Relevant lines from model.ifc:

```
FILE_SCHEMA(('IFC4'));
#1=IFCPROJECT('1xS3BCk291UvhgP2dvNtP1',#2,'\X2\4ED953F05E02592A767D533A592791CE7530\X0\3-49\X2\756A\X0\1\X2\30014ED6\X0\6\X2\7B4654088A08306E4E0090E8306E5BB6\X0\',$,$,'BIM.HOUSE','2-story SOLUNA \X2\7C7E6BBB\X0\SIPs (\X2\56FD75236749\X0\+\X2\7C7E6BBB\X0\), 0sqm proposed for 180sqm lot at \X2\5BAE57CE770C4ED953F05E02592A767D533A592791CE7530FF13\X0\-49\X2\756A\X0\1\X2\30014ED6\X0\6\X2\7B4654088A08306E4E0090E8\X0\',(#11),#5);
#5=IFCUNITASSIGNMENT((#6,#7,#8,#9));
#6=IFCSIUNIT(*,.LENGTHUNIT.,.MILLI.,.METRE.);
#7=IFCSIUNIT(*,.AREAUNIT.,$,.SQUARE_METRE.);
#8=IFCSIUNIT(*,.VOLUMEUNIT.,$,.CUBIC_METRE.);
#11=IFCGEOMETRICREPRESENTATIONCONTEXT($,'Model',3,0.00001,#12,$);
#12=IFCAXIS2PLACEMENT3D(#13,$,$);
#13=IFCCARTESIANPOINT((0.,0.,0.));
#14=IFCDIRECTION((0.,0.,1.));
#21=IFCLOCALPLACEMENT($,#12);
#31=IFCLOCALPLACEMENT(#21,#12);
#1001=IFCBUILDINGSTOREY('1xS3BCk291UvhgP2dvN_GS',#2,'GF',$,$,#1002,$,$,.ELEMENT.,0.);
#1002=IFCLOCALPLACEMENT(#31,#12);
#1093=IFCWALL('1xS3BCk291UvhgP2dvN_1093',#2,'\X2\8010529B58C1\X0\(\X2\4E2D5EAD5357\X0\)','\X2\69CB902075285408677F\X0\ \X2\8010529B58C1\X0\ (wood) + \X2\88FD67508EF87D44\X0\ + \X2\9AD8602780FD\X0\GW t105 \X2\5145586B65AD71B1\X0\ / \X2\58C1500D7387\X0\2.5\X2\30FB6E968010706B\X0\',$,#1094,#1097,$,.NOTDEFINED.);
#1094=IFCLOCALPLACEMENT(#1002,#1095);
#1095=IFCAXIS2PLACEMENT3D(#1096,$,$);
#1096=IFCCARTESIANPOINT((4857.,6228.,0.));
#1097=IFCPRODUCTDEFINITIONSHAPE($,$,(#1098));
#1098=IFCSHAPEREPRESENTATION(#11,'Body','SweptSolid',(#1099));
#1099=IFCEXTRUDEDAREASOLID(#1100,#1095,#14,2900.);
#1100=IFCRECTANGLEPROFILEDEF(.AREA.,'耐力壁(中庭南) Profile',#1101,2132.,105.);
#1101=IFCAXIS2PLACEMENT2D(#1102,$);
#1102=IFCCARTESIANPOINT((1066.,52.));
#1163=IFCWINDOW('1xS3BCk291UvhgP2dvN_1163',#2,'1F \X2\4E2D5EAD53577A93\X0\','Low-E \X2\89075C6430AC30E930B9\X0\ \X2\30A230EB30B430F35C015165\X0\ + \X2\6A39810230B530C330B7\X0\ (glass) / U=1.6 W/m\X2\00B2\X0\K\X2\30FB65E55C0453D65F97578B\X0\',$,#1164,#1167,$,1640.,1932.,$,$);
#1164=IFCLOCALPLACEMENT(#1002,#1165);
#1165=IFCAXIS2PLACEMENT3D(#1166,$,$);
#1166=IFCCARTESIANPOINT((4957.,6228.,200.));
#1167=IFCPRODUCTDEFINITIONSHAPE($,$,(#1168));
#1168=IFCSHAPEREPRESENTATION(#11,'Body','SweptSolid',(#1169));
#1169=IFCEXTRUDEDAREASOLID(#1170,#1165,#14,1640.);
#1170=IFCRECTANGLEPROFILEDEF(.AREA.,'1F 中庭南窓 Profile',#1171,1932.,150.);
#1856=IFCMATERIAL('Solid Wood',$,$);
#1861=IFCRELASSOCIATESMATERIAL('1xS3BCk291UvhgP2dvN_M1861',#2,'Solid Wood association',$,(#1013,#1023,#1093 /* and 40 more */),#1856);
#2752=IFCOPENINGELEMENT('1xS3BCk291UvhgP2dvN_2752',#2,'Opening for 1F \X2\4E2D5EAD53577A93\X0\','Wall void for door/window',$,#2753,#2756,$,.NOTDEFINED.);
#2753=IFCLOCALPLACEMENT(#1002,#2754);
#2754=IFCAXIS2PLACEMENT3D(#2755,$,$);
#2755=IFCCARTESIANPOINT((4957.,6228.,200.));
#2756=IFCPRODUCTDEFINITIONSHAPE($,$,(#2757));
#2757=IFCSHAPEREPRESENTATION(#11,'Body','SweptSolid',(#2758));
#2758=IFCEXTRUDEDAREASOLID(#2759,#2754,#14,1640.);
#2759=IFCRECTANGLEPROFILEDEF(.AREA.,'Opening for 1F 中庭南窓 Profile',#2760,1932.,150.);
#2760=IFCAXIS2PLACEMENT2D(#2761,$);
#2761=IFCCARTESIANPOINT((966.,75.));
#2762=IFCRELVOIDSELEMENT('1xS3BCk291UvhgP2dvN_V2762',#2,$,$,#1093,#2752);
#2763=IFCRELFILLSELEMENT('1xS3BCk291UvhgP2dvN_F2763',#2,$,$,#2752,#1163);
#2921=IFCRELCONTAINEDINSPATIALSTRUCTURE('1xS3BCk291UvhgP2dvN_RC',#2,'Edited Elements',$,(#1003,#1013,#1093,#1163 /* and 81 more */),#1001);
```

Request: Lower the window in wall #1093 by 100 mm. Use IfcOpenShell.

```python
import numpy as np
import ifcopenshell
import ifcopenshell.api.geometry
import ifcopenshell.util.placement
import ifcopenshell.util.unit

model = ifcopenshell.open("model.ifc")
unit_scale = ifcopenshell.util.unit.calculate_unit_scale(model)

window = model.by_id(1163)
opening = window.FillsVoids[0].RelatingOpeningElement
dz = -0.1 / unit_scale

shift = np.array([0.0, 0.0, dz])
# The window is not placed relative to its opening, so move both.
for product in (opening, window):
    matrix = ifcopenshell.util.placement.get_local_placement(product.ObjectPlacement)
    matrix[:3, 3] += shift
    ifcopenshell.api.geometry.edit_object_placement(model, product=product, matrix=matrix, is_si=False)

print(f"moved by {dz * unit_scale:+.3f} m")

model.write("model_updated.ifc")
```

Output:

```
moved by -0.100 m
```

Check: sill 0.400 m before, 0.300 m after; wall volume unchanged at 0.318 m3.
